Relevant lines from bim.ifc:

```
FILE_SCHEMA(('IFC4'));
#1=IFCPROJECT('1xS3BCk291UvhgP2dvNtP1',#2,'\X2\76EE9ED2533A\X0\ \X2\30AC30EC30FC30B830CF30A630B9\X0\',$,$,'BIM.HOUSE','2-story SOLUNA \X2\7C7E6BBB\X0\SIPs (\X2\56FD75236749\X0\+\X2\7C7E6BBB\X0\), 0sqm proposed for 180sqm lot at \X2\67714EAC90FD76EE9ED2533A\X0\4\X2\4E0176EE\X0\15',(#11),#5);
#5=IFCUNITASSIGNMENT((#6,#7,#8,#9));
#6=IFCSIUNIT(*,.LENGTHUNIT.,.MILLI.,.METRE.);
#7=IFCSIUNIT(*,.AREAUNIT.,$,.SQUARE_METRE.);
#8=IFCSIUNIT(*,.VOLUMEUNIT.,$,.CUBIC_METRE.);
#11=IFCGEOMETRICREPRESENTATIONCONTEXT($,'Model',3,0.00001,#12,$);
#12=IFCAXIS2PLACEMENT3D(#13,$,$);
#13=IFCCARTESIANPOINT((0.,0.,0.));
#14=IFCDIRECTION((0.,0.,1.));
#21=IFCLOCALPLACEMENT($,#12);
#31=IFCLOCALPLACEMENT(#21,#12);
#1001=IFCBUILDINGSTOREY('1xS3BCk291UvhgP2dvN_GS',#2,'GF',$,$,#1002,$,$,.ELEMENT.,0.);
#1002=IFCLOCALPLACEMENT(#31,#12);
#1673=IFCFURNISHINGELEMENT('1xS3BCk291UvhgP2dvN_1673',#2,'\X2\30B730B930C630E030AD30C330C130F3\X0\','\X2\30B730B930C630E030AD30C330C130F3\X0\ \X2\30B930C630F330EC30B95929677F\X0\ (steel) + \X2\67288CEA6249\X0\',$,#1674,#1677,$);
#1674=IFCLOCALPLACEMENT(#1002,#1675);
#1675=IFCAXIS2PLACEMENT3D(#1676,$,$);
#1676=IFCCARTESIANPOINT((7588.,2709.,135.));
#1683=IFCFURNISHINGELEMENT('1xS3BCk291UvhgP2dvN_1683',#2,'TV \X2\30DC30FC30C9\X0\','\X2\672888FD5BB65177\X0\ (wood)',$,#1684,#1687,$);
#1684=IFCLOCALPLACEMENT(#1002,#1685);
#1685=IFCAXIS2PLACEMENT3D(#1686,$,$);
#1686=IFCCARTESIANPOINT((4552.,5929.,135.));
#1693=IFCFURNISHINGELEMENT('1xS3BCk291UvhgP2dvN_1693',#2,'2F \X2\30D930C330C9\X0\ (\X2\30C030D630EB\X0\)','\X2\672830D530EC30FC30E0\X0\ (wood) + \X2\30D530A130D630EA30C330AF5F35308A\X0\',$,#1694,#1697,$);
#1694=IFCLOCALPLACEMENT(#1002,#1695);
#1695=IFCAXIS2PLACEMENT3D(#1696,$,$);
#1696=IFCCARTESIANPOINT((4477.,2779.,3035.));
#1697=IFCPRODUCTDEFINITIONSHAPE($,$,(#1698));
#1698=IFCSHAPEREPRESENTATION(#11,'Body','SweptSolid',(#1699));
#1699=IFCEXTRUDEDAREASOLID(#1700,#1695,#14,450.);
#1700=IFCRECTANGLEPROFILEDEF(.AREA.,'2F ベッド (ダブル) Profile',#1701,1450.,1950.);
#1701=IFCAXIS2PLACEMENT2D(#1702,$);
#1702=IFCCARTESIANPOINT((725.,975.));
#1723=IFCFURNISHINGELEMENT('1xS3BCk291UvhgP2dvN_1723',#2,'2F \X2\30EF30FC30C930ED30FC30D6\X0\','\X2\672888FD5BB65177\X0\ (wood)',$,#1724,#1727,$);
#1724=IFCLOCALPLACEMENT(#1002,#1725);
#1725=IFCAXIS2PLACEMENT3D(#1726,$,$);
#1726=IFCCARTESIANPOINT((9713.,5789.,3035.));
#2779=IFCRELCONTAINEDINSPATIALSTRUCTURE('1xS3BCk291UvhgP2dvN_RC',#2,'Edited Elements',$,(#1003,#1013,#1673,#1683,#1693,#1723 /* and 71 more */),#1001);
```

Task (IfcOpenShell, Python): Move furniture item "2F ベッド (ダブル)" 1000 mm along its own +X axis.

```python
import ifcopenshell
import ifcopenshell.api.geometry
import ifcopenshell.util.placement

model = ifcopenshell.open("bim.ifc")

item = model.by_guid("1xS3BCk291UvhgP2dvN_1693")
matrix = ifcopenshell.util.placement.get_local_placement(item.ObjectPlacement)
matrix[:3, 3] += matrix[:3, 0] * 1000.0
ifcopenshell.api.geometry.edit_object_placement(model, product=item, matrix=matrix, is_si=False)

print(ifcopenshell.util.placement.get_local_placement(item.ObjectPlacement).round(3) + 0.0)

model.write("bim_updated.ifc")
```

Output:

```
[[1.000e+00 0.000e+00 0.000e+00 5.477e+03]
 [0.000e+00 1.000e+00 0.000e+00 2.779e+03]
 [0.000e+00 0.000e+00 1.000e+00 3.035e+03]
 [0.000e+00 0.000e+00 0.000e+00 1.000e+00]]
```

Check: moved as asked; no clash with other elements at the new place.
